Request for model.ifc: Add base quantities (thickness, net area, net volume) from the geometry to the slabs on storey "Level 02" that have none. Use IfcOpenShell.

First a look at what the model holds.

```python
import ifcopenshell
import ifcopenshell.util.element
import ifcopenshell.util.unit

model = ifcopenshell.open("model.ifc")
print(model.schema)
for unit_type in ("LENGTHUNIT", "AREAUNIT", "VOLUMEUNIT"):
    print(unit_type, ifcopenshell.util.unit.calculate_unit_scale(model, unit_type))
storey = next(s for s in model.by_type("IfcBuildingStorey") if s.Name == "Level 02")
slabs = [e for e in ifcopenshell.util.element.get_decomposition(storey) if e.is_a("IfcSlab")]
for e in sorted(slabs, key=lambda e: e.id()):
    print(e.id(), e.is_a(), e.Name, list(ifcopenshell.util.element.get_psets(e, qtos_only=True)), sep=" | ")
```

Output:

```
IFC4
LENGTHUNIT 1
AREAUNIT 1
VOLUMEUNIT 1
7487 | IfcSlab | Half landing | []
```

```python
import ifcopenshell
import ifcopenshell.api.pset
import ifcopenshell.geom
import ifcopenshell.util.element
import ifcopenshell.util.shape
import ifcopenshell.util.unit

model = ifcopenshell.open("model.ifc")
unit_scale = ifcopenshell.util.unit.calculate_unit_scale(model)
area_scale = ifcopenshell.util.unit.calculate_unit_scale(model, "AREAUNIT")
volume_scale = ifcopenshell.util.unit.calculate_unit_scale(model, "VOLUMEUNIT")
settings = ifcopenshell.geom.settings()

storey = next(s for s in model.by_type("IfcBuildingStorey") if s.Name == "Level 02")
slabs = [e for e in ifcopenshell.util.element.get_decomposition(storey) if e.is_a("IfcSlab")]

for e in sorted(slabs, key=lambda e: e.id()):
    if ifcopenshell.util.element.get_psets(e, qtos_only=True, should_inherit=False):
        continue
    # Geometry comes back in metres, in the element's own axes.
    shape = ifcopenshell.geom.create_shape(settings, e)
    values = {
        "Width": ifcopenshell.util.shape.get_z(shape.geometry) / unit_scale,
        "NetArea": ifcopenshell.util.shape.get_footprint_area(shape.geometry) / area_scale,
        "NetVolume": ifcopenshell.util.shape.get_volume(shape.geometry) / volume_scale,
    }
    qto = ifcopenshell.api.pset.add_qto(model, product=e, name="Qto_SlabBaseQuantities")
    ifcopenshell.api.pset.edit_qto(model, qto=qto, properties=values)
    print(e.id(), {k: round(v, 3) for k, v in values.items()})

model.write("model-out.ifc")
```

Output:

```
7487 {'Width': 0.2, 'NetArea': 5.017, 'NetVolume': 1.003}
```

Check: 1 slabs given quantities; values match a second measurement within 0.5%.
